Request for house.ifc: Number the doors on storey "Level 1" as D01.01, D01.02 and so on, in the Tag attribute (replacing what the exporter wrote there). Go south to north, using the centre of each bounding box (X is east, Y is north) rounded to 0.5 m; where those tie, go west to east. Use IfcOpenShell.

First a look at what the model holds.

```python
import ifcopenshell
import ifcopenshell.util.element
import ifcopenshell.util.placement

model = ifcopenshell.open("house.ifc")
print(model.schema)
storey = next(s for s in model.by_type("IfcBuildingStorey") if s.Name == "Level 1")
doors = [e for e in ifcopenshell.util.element.get_decomposition(storey) if e.is_a("IfcDoor")]
for e in sorted(doors, key=lambda e: e.id()):
    origin = ifcopenshell.util.placement.get_local_placement(e.ObjectPlacement)[:3, 3]
    print(e.id(), e.Tag, e.Name, origin.round(2) + 0.0, sep=" | ")
```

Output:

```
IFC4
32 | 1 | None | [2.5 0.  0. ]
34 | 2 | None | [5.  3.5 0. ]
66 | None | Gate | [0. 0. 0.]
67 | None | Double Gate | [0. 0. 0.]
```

```python
import ifcopenshell
import ifcopenshell.geom
import ifcopenshell.util.element
import ifcopenshell.util.shape

model = ifcopenshell.open("house.ifc")
settings = ifcopenshell.geom.settings()
settings.set("use-world-coords", True)


def centre(element):
    shape = ifcopenshell.geom.create_shape(settings, element)
    return ifcopenshell.util.shape.get_bbox_centroid(shape.geometry)


storey = next(s for s in model.by_type("IfcBuildingStorey") if s.Name == "Level 1")
doors = [e for e in ifcopenshell.util.element.get_decomposition(storey) if e.is_a("IfcDoor")]

# Insertion points can sit at a corner or the storey origin, so sort by the geometry (in metres).
centres = {e: centre(e) for e in doors}
doors.sort(key=lambda e: (round(centres[e][1] / 0.5), centres[e][0]))

for i, e in enumerate(doors, start=1):
    number = f"D01.{i:02d}"
    e.Tag = number
    print(e.id(), number)

model.write("house_edited.ifc")
```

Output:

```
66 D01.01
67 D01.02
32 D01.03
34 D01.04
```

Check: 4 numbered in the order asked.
